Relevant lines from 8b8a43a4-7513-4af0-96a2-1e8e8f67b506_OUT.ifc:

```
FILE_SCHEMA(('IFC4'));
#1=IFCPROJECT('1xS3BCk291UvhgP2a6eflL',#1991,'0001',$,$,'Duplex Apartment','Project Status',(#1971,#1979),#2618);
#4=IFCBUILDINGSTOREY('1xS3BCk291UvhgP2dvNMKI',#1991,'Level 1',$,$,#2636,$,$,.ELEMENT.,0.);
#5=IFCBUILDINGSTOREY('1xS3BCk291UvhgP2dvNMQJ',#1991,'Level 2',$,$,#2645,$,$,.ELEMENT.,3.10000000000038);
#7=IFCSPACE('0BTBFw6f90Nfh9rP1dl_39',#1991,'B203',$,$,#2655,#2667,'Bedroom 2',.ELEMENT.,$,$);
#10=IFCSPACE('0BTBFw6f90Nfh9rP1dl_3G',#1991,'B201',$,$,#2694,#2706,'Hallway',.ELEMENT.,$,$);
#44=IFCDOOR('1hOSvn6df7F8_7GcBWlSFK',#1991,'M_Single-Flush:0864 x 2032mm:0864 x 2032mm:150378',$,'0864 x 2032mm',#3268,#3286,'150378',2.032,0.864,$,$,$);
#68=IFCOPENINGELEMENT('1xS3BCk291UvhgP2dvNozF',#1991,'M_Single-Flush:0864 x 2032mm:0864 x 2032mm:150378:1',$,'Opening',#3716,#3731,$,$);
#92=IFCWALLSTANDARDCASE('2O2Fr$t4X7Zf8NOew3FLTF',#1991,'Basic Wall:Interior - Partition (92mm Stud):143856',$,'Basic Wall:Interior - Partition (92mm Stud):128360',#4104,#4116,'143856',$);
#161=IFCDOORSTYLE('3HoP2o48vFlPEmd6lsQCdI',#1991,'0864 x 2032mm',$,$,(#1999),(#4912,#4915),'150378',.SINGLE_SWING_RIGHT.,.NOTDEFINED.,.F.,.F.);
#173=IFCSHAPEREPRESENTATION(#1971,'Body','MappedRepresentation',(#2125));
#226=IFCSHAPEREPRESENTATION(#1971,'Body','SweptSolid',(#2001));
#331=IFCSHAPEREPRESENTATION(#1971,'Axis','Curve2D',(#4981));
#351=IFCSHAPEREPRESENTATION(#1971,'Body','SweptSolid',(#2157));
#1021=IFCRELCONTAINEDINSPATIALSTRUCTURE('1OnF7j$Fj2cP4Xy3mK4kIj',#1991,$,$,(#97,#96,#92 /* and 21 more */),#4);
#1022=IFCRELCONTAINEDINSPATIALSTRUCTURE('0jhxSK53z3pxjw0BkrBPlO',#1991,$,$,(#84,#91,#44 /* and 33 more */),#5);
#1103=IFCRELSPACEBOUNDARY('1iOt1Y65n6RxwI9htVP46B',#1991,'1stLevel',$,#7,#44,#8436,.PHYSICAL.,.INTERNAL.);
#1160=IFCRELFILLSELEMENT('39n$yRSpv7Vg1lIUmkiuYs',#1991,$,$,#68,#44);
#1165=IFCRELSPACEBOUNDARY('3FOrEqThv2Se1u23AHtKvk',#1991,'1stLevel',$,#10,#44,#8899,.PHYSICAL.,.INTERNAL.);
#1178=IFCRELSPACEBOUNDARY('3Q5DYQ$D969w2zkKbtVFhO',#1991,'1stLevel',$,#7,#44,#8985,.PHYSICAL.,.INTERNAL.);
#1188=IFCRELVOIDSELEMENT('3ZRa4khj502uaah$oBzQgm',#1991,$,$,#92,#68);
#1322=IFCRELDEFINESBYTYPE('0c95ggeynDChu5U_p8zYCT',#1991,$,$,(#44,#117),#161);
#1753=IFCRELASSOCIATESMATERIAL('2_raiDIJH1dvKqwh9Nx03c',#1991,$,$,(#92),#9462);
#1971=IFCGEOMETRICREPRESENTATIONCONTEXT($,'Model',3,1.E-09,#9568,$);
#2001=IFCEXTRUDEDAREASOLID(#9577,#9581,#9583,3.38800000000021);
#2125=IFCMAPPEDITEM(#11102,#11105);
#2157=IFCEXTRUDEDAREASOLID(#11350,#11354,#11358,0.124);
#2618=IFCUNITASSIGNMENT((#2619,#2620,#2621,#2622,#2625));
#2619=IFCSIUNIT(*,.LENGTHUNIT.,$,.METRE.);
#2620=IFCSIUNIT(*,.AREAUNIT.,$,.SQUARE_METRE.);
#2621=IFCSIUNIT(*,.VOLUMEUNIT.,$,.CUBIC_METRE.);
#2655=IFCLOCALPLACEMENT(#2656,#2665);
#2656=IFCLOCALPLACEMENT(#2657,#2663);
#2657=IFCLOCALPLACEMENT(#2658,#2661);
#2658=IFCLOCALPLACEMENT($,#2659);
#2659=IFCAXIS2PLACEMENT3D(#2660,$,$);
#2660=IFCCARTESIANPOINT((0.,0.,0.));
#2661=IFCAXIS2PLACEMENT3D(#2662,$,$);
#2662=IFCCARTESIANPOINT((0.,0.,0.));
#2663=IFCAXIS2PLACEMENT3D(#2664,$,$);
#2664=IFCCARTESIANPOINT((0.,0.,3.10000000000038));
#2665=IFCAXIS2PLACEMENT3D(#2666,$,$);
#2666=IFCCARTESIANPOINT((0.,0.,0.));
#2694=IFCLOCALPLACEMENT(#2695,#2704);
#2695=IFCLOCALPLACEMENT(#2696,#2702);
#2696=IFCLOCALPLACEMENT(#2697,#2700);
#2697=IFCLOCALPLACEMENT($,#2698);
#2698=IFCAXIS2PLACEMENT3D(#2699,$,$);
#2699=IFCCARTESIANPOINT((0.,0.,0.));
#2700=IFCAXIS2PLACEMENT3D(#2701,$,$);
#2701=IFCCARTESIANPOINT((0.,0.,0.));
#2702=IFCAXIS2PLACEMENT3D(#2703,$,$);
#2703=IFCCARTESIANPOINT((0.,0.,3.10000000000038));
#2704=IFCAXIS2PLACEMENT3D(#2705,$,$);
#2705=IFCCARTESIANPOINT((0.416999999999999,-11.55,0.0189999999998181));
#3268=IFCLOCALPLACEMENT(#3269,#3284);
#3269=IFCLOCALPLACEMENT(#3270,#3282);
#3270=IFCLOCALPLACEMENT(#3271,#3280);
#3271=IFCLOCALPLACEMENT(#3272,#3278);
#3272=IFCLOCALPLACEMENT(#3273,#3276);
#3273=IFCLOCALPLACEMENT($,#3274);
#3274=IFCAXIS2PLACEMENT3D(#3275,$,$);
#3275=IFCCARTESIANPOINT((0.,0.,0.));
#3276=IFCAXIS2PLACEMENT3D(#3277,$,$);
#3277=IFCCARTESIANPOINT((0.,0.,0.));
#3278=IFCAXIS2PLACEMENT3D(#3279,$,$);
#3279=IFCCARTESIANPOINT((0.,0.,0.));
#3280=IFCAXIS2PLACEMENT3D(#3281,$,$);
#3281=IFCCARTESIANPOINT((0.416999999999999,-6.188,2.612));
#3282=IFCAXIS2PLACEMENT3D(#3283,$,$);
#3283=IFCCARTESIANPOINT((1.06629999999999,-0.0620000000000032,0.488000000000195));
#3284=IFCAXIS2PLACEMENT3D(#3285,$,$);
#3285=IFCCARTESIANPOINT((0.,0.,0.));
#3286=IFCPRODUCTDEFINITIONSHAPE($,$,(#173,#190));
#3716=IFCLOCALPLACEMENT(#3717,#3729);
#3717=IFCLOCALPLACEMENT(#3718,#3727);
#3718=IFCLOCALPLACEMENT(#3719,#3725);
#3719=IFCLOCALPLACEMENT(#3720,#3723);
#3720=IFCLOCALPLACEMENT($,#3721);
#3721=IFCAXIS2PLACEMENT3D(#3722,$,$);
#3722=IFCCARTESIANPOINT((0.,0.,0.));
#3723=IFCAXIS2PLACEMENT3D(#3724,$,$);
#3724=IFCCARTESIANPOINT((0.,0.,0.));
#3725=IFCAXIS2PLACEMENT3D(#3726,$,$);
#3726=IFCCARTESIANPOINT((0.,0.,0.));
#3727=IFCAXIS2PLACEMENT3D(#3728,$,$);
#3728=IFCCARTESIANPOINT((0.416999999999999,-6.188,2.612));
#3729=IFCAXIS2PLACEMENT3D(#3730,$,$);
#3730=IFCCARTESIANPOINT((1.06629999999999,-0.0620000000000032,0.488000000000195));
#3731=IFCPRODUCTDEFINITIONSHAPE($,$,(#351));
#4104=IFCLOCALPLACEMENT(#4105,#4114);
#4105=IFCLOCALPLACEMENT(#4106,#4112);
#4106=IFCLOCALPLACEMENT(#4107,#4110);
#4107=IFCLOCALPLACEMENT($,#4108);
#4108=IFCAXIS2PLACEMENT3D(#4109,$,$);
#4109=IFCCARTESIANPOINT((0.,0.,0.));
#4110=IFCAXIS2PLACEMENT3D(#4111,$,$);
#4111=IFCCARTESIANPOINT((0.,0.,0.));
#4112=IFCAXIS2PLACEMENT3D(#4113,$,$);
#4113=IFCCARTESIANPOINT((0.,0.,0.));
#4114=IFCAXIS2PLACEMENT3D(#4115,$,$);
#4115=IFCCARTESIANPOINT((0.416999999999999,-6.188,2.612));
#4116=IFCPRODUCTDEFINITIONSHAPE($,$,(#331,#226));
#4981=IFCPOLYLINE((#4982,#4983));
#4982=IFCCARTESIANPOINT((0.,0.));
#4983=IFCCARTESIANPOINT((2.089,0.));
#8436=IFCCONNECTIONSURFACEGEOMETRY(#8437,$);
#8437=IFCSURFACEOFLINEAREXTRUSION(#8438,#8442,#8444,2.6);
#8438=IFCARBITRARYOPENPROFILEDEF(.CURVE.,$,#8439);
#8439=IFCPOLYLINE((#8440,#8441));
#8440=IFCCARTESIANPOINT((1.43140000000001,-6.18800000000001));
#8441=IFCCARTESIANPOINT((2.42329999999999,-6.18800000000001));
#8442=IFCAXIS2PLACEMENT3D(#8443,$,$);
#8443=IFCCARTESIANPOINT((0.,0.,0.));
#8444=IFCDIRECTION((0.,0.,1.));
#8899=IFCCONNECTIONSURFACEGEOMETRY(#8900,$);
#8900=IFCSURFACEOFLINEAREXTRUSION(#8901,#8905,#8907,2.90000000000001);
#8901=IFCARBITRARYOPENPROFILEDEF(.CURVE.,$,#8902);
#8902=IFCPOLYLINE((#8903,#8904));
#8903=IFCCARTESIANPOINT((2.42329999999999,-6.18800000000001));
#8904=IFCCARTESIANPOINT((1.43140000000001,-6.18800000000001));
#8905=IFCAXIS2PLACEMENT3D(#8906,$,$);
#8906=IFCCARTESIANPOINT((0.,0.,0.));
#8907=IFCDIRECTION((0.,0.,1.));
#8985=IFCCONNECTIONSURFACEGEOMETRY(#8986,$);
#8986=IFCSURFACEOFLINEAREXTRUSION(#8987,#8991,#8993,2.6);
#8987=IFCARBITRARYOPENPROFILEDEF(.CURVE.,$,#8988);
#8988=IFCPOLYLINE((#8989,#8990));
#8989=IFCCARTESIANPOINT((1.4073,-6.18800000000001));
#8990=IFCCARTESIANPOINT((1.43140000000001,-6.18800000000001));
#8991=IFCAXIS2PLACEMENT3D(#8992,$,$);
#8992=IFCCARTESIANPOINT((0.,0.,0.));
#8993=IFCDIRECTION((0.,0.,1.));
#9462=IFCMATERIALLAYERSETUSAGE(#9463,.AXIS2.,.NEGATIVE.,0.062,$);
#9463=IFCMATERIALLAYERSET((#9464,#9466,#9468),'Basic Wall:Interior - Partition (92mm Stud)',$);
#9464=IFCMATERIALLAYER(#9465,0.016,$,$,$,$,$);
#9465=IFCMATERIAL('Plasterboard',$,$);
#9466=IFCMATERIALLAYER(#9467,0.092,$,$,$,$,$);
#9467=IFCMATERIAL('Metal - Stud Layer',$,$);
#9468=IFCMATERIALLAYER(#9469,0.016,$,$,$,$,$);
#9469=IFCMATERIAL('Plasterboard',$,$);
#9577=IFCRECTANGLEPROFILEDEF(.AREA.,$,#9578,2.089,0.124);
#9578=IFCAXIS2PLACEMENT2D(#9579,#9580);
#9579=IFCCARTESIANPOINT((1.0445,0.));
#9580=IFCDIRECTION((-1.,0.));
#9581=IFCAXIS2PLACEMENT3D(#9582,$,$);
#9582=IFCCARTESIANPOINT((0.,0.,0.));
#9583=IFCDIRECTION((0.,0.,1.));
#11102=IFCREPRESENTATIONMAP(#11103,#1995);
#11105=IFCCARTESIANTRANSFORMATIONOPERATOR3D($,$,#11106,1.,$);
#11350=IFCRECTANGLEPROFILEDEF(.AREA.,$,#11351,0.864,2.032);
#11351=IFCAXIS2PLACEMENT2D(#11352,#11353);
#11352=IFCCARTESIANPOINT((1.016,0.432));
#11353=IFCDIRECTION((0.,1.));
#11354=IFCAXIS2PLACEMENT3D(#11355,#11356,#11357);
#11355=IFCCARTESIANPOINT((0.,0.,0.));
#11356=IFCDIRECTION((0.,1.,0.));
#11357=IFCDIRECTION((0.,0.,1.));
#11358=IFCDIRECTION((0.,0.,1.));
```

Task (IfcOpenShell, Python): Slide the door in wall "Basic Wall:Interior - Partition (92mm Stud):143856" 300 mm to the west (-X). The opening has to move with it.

```python
import numpy as np
import ifcopenshell
import ifcopenshell.api.geometry
import ifcopenshell.util.placement
import ifcopenshell.util.unit

model = ifcopenshell.open("8b8a43a4-7513-4af0-96a2-1e8e8f67b506_OUT.ifc")
unit_scale = ifcopenshell.util.unit.calculate_unit_scale(model)

door = model.by_id(44)
opening = door.FillsVoids[0].RelatingOpeningElement
wall = opening.VoidsElements[0].RelatingBuildingElement

wall_matrix = ifcopenshell.util.placement.get_local_placement(wall.ObjectPlacement)
shift = wall_matrix[:3, 0] * -0.3 / unit_scale
before = ifcopenshell.util.placement.get_local_placement(door.ObjectPlacement)[:3, 3].copy()

# The door is not placed relative to its opening, so move both.
for product in (opening, door):
    matrix = ifcopenshell.util.placement.get_local_placement(product.ObjectPlacement)
    matrix[:3, 3] += shift
    ifcopenshell.api.geometry.edit_object_placement(model, product=product, matrix=matrix, is_si=False)

# Space boundary surfaces are stored in each space's coordinates; move them too.
for rel in door.ProvidesBoundaries:
    if not rel.ConnectionGeometry:
        continue
    surface = rel.ConnectionGeometry.SurfaceOnRelatingElement
    space_matrix = ifcopenshell.util.placement.get_local_placement(rel.RelatingSpace.ObjectPlacement)
    point = np.array(surface.Position.Location.Coordinates) + space_matrix[:3, :3].T @ shift
    surface.Position = model.createIfcAxis2Placement3D(
        model.createIfcCartesianPoint(point.tolist()), surface.Position.Axis, surface.Position.RefDirection
    )

after = ifcopenshell.util.placement.get_local_placement(door.ObjectPlacement)[:3, 3]
print("door moved by", (after - before).round(3) + 0.0)

model.write("8b8a43a4-7513-4af0-96a2-1e8e8f67b506_OUT_updated.ifc")
```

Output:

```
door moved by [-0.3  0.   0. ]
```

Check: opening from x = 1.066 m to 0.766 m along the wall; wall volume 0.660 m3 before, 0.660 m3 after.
